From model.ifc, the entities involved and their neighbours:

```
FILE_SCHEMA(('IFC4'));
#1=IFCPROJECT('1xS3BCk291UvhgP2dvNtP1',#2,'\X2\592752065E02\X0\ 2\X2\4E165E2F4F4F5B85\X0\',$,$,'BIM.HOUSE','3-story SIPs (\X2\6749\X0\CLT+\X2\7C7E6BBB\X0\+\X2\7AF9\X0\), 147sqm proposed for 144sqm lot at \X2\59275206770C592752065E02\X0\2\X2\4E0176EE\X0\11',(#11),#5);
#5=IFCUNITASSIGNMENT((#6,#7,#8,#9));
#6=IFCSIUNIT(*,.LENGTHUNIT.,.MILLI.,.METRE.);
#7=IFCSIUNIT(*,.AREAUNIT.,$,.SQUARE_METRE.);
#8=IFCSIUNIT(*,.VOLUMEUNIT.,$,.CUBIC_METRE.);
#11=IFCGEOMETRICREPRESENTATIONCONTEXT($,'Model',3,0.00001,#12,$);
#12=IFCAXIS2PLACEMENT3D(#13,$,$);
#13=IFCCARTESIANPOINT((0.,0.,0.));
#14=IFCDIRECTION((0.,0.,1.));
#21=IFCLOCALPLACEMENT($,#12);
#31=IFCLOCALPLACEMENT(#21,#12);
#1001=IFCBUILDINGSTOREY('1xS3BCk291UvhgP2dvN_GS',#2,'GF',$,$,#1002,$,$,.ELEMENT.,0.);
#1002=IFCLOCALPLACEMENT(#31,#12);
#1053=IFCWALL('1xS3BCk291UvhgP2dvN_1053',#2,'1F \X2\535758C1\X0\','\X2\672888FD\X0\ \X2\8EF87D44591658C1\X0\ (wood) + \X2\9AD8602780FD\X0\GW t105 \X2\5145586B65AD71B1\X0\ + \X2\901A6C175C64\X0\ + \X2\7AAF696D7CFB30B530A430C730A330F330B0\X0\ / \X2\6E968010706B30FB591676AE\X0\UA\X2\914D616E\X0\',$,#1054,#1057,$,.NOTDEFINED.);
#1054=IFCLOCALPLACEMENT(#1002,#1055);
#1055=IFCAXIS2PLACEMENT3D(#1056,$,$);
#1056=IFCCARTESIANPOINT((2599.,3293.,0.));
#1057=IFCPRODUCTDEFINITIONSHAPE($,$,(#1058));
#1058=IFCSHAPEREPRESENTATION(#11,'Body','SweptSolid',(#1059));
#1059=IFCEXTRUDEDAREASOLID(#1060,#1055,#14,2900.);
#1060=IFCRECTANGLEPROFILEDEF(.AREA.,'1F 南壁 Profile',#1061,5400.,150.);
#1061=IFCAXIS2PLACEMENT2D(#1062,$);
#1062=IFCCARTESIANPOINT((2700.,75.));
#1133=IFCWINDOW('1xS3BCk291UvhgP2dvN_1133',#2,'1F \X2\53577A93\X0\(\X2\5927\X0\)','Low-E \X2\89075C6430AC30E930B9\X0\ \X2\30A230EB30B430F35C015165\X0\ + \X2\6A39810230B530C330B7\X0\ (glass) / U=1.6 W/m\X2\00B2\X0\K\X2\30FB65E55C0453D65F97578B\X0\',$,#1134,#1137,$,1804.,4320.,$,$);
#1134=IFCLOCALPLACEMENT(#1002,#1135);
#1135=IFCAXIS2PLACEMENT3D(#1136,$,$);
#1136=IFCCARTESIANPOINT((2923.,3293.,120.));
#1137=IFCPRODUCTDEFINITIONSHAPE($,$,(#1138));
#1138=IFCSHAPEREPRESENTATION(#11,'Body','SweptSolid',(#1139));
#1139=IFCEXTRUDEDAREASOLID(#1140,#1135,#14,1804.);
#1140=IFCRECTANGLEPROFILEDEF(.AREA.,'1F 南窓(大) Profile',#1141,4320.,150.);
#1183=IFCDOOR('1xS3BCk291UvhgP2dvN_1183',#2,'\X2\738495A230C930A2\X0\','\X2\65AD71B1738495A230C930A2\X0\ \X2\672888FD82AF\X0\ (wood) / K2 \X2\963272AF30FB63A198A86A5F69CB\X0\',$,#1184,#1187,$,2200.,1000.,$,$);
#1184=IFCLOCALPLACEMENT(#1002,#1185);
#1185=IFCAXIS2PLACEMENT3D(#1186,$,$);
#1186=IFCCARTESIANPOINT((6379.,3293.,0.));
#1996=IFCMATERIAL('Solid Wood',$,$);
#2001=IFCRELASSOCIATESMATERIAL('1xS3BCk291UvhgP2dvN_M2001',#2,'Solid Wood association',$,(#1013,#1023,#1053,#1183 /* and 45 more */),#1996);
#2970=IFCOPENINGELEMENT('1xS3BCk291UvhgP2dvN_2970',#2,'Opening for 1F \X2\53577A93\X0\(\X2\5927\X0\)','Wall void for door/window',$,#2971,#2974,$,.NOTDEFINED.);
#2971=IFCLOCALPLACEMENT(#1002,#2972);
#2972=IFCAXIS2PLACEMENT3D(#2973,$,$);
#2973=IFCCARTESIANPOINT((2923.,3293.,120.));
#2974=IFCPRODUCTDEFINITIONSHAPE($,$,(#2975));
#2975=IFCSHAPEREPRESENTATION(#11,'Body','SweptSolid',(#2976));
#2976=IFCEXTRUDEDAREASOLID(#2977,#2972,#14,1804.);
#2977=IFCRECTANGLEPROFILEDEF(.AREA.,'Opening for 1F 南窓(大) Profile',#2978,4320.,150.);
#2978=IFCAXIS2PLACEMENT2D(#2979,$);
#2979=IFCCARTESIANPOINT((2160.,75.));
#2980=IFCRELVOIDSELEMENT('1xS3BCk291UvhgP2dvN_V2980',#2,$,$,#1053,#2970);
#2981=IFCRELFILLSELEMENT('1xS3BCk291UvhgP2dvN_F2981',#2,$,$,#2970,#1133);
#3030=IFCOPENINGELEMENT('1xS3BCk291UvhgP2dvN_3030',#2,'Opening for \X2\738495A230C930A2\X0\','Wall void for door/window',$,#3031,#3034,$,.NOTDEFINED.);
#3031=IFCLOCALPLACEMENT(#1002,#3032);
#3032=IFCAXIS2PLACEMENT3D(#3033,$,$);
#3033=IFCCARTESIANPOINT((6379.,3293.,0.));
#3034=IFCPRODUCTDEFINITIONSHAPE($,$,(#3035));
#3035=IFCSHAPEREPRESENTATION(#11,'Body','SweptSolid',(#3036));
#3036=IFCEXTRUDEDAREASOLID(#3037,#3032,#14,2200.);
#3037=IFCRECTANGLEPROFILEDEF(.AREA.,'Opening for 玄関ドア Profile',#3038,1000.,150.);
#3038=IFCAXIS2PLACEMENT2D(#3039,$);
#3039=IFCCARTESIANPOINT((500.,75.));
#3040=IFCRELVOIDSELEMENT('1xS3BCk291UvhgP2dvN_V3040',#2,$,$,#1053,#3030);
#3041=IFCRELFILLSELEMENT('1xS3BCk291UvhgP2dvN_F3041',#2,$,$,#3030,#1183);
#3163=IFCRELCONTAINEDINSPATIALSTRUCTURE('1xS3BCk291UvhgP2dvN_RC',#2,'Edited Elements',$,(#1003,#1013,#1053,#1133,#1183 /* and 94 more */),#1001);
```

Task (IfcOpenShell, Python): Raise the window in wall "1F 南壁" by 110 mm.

```python
import numpy as np
import ifcopenshell
import ifcopenshell.api.geometry
import ifcopenshell.util.placement
import ifcopenshell.util.unit

model = ifcopenshell.open("model.ifc")
unit_scale = ifcopenshell.util.unit.calculate_unit_scale(model)

window = model.by_guid("1xS3BCk291UvhgP2dvN_1133")
opening = window.FillsVoids[0].RelatingOpeningElement
dz = 0.11 / unit_scale

shift = np.array([0.0, 0.0, dz])
# The window is not placed relative to its opening, so move both.
for product in (opening, window):
    matrix = ifcopenshell.util.placement.get_local_placement(product.ObjectPlacement)
    matrix[:3, 3] += shift
    ifcopenshell.api.geometry.edit_object_placement(model, product=product, matrix=matrix, is_si=False)

print(f"moved by {dz * unit_scale:+.3f} m")

model.write("model_v2.ifc")
```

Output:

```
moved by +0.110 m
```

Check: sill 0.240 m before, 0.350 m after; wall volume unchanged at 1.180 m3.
